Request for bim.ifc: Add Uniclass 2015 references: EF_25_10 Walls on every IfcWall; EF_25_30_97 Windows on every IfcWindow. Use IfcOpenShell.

First a look at what the model holds.

```python
import ifcopenshell

model = ifcopenshell.open("bim.ifc")
print(model.schema)
print("classifications:", [c.Name for c in model.by_type("IfcClassification")])
for ifc_class in ("IfcDoor", "IfcRoof", "IfcStair", "IfcWall", "IfcWindow"):
    print(ifc_class, len(model.by_type(ifc_class)))
```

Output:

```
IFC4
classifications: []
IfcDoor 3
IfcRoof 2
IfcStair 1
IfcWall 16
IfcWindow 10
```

```python
import ifcopenshell
import ifcopenshell.api.classification

model = ifcopenshell.open("bim.ifc")

system = ifcopenshell.api.classification.add_classification(model, classification="Uniclass 2015")

codes = {
    "IfcWall": ("EF_25_10", "Walls"),
    "IfcWindow": ("EF_25_30_97", "Windows"),
}
for ifc_class, (code, name) in codes.items():
    products = model.by_type(ifc_class)
    ifcopenshell.api.classification.add_reference(
        model, products=products, classification=system, identification=code, name=name
    )
    print(code, len(products))

model.write("bim_rev.ifc")
```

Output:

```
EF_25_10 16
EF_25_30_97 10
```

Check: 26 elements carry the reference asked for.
